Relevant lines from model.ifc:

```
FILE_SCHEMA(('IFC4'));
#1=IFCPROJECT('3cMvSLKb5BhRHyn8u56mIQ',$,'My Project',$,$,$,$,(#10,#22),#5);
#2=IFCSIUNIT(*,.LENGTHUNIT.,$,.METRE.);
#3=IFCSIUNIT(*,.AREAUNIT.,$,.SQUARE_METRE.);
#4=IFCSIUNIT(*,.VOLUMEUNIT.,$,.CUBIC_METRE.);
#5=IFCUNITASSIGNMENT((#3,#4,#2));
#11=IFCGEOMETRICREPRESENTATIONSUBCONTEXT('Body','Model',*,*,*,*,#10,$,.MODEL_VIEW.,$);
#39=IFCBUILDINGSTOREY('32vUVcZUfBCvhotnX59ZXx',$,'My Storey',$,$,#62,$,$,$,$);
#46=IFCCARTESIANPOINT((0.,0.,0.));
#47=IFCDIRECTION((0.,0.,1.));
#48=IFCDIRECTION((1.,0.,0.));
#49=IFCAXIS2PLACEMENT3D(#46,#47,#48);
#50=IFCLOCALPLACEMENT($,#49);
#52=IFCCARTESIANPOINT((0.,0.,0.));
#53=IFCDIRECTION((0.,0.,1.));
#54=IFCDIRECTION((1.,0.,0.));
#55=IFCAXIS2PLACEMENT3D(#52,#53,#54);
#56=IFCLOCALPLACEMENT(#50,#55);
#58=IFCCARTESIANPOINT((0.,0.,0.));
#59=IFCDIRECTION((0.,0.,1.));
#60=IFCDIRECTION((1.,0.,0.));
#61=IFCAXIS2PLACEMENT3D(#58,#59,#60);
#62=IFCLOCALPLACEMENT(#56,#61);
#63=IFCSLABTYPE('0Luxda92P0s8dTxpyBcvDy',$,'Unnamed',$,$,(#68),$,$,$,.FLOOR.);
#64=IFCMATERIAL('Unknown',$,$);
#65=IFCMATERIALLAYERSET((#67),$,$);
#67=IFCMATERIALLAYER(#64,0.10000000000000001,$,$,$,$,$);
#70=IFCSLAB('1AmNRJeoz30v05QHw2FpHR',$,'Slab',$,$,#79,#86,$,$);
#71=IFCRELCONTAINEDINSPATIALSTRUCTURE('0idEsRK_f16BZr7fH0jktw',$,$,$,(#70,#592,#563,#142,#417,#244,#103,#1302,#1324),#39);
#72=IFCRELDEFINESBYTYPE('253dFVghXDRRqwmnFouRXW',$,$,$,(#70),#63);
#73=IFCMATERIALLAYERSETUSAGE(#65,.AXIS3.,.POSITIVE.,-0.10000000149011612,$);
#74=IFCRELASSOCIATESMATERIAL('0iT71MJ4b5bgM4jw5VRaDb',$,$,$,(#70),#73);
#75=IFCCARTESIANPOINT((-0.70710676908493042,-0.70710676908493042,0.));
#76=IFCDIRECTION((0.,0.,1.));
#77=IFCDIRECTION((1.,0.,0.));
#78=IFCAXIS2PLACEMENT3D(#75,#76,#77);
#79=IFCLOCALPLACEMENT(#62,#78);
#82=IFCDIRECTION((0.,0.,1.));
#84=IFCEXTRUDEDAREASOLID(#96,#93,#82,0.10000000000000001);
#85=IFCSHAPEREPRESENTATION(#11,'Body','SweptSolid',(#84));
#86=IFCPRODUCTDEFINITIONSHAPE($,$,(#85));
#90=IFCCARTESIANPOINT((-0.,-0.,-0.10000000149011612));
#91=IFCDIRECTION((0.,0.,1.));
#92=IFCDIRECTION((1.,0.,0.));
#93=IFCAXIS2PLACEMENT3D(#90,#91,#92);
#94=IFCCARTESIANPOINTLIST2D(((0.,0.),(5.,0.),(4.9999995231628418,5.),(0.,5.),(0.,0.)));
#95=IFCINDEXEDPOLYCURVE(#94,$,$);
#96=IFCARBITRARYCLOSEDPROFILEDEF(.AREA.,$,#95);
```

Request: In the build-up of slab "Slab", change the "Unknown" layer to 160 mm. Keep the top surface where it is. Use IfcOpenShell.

```python
import ifcopenshell
import ifcopenshell.util.element
import ifcopenshell.util.representation
import ifcopenshell.util.unit

model = ifcopenshell.open("model.ifc")
unit_scale = ifcopenshell.util.unit.calculate_unit_scale(model)

layer_set = model.by_id(65)
layer = next(l for l in layer_set.MaterialLayers if l.Material and l.Material.Name == "Unknown")
change = 0.16 / unit_scale - layer.LayerThickness
layer.LayerThickness += change

# Geometry does not follow the layer set by itself.
slabs = [e for e in ifcopenshell.util.element.get_elements_by_material(model, layer_set) if e.is_a("IfcSlab")]
for slab in sorted(slabs, key=lambda e: e.id()):
    body = ifcopenshell.util.representation.get_representation(slab, "Model", "Body")
    solid = body.Items[0]
    old_depth = solid.Depth
    solid.Depth += change
    # Extruded upwards: lower the start of the extrusion so the top stays.
    x, y, z = solid.Position.Location.Coordinates
    solid.Position.Location = model.createIfcCartesianPoint((x, y, z - change))
    print(slab.id(), f"{old_depth:g} -> {solid.Depth:g}")

# The layers are counted up from the underside, which has moved.
for usage in {ifcopenshell.util.element.get_material(slab) for slab in slabs}:
    usage.OffsetFromReferenceLine -= change

model.write("model_updated.ifc")
```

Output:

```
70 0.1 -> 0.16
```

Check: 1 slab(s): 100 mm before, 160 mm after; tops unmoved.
